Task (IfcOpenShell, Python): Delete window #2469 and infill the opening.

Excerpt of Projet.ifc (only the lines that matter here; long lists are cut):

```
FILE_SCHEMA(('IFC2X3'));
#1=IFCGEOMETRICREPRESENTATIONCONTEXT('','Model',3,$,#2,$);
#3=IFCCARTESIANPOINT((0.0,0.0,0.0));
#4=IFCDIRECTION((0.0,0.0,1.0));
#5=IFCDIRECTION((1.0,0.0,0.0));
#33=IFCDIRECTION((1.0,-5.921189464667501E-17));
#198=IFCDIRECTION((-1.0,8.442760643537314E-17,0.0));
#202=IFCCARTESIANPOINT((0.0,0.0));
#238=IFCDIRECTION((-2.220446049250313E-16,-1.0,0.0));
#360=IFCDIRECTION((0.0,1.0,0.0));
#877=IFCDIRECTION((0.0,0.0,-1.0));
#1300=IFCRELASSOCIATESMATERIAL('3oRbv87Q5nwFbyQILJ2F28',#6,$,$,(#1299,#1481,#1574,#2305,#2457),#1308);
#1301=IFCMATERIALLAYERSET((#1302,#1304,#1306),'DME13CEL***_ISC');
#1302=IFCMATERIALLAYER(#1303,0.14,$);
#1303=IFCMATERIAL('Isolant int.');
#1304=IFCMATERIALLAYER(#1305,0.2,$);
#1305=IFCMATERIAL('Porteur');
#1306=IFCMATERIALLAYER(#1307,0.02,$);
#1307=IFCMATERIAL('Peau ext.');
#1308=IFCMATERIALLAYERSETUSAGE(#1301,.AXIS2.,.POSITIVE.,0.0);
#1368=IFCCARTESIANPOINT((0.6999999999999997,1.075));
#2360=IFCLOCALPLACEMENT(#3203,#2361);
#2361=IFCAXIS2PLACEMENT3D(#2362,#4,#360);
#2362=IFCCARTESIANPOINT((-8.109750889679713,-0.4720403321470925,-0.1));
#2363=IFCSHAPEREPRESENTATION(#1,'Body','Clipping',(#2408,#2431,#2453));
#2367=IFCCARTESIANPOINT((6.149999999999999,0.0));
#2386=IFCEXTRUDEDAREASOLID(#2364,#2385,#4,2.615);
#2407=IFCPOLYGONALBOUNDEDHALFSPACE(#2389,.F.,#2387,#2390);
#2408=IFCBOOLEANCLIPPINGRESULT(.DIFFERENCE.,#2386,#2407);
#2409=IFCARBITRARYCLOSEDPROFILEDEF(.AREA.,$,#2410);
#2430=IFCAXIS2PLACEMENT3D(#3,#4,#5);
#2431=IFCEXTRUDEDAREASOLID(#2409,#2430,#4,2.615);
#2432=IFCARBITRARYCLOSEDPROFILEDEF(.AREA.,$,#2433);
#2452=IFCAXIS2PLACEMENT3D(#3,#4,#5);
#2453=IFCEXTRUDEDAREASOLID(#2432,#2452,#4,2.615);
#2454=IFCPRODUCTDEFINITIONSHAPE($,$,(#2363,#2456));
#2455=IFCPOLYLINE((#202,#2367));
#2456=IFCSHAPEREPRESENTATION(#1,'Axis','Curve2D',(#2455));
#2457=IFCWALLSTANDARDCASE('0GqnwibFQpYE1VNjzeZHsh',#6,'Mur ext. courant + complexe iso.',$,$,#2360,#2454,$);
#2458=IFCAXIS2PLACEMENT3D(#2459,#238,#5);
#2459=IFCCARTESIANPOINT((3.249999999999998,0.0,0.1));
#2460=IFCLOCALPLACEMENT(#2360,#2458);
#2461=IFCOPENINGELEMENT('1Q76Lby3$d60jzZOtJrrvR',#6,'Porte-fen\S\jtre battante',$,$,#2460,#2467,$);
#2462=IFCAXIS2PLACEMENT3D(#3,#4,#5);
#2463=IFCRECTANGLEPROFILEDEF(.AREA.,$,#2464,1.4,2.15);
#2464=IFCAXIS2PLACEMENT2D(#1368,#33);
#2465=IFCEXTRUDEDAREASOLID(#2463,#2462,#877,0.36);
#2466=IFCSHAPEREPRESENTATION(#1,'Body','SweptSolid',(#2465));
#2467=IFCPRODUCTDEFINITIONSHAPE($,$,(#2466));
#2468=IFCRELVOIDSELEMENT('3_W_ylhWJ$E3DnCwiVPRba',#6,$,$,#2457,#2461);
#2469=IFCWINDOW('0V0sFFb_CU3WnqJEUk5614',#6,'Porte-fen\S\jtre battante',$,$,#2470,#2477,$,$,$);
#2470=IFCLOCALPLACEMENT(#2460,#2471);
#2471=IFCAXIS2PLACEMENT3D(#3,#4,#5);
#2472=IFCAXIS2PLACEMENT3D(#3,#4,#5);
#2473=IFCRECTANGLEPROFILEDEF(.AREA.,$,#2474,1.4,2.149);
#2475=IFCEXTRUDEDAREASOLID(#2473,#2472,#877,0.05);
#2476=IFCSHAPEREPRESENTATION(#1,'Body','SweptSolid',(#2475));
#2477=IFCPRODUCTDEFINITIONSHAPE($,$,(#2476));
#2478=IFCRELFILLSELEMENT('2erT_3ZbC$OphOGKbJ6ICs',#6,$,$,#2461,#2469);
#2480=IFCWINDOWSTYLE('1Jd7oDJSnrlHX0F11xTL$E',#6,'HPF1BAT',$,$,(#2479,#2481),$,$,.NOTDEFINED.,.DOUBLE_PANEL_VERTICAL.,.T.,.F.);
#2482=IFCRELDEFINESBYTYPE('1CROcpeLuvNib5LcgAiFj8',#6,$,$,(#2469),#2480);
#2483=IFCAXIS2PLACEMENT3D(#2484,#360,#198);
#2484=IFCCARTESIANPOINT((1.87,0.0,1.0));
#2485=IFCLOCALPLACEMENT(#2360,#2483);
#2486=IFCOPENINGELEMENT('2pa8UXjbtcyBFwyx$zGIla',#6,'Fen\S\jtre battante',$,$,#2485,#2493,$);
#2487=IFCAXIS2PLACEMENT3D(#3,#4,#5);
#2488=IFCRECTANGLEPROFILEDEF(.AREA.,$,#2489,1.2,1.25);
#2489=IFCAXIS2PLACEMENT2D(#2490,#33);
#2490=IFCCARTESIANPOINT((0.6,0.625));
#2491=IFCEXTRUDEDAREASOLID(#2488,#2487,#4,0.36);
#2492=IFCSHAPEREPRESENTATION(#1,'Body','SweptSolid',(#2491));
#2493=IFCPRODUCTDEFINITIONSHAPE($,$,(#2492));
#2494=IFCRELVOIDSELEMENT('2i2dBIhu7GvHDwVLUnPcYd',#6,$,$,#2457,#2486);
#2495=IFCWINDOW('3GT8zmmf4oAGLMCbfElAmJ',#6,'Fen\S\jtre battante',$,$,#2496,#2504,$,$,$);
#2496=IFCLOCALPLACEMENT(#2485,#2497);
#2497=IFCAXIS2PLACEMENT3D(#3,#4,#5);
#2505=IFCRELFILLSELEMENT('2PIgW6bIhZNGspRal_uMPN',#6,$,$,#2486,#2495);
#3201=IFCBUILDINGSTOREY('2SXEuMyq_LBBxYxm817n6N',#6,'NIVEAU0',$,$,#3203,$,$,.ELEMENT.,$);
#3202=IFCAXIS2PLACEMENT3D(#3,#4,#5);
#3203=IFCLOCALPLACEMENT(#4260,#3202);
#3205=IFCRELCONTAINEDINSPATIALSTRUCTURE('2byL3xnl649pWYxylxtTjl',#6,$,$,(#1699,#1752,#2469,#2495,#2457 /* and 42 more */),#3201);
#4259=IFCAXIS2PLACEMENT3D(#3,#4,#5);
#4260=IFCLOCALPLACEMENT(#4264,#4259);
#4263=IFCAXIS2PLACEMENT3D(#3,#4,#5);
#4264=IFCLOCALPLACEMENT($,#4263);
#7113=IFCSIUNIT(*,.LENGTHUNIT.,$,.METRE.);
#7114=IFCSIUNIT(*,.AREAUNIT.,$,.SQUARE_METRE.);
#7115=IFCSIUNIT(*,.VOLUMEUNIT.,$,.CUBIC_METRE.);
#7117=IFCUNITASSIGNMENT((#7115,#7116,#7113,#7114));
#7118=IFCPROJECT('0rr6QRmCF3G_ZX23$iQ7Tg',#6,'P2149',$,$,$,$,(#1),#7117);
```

```python
import ifcopenshell
import ifcopenshell.api.feature
import ifcopenshell.api.root
import ifcopenshell.geom
import ifcopenshell.util.shape

model = ifcopenshell.open("Projet.ifc")
settings = ifcopenshell.geom.settings()


def volume(element):
    """Net volume in cubic metres, openings subtracted."""
    shape = ifcopenshell.geom.create_shape(settings, element)
    return ifcopenshell.util.shape.get_volume(shape.geometry)


window = model.by_id(2469)
opening = window.FillsVoids[0].RelatingOpeningElement
wall = opening.VoidsElements[0].RelatingBuildingElement
before = volume(wall)

ifcopenshell.api.root.remove_product(model, product=window)
ifcopenshell.api.feature.remove_feature(model, feature=opening)

after = volume(wall)

print(f"wall volume {before:.3f} -> {after:.3f} m3")

model.write("Projet_rev.ifc")
```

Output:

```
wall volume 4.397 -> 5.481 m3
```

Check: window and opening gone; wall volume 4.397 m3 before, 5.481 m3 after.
